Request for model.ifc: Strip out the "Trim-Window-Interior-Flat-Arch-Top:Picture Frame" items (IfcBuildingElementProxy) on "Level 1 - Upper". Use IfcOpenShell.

First a look at what the model holds.

```python
import ifcopenshell
import ifcopenshell.util.element

model = ifcopenshell.open("model.ifc")
print(model.schema)
storey = next(s for s in model.by_type("IfcBuildingStorey") if s.Name == "Level 1 - Upper")
proxies = [e for e in ifcopenshell.util.element.get_decomposition(storey) if e.is_a("IfcBuildingElementProxy")]
seen = {}
for e in proxies:
    element_type = ifcopenshell.util.element.get_type(e)
    name = element_type.Name if element_type not in (None, e) else None
    seen[name] = seen.get(name, 0) + 1
for name, count in sorted(seen.items(), key=str):
    print(count, "x", name)
```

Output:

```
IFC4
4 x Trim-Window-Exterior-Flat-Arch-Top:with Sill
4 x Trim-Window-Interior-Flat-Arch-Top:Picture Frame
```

```python
import ifcopenshell
import ifcopenshell.api.root
import ifcopenshell.util.element

model = ifcopenshell.open("model.ifc")

storey = next(s for s in model.by_type("IfcBuildingStorey") if s.Name == "Level 1 - Upper")
proxies = [e for e in ifcopenshell.util.element.get_decomposition(storey) if e.is_a("IfcBuildingElementProxy")]
targets = [e for e in proxies if (t := ifcopenshell.util.element.get_type(e)) not in (None, e) and t.Name == "Trim-Window-Interior-Flat-Arch-Top:Picture Frame"]

for e in targets:
    ifcopenshell.api.root.remove_product(model, product=e)
print(len(targets), "removed")

model.write("model-out.ifc")
```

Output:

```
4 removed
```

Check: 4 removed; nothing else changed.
